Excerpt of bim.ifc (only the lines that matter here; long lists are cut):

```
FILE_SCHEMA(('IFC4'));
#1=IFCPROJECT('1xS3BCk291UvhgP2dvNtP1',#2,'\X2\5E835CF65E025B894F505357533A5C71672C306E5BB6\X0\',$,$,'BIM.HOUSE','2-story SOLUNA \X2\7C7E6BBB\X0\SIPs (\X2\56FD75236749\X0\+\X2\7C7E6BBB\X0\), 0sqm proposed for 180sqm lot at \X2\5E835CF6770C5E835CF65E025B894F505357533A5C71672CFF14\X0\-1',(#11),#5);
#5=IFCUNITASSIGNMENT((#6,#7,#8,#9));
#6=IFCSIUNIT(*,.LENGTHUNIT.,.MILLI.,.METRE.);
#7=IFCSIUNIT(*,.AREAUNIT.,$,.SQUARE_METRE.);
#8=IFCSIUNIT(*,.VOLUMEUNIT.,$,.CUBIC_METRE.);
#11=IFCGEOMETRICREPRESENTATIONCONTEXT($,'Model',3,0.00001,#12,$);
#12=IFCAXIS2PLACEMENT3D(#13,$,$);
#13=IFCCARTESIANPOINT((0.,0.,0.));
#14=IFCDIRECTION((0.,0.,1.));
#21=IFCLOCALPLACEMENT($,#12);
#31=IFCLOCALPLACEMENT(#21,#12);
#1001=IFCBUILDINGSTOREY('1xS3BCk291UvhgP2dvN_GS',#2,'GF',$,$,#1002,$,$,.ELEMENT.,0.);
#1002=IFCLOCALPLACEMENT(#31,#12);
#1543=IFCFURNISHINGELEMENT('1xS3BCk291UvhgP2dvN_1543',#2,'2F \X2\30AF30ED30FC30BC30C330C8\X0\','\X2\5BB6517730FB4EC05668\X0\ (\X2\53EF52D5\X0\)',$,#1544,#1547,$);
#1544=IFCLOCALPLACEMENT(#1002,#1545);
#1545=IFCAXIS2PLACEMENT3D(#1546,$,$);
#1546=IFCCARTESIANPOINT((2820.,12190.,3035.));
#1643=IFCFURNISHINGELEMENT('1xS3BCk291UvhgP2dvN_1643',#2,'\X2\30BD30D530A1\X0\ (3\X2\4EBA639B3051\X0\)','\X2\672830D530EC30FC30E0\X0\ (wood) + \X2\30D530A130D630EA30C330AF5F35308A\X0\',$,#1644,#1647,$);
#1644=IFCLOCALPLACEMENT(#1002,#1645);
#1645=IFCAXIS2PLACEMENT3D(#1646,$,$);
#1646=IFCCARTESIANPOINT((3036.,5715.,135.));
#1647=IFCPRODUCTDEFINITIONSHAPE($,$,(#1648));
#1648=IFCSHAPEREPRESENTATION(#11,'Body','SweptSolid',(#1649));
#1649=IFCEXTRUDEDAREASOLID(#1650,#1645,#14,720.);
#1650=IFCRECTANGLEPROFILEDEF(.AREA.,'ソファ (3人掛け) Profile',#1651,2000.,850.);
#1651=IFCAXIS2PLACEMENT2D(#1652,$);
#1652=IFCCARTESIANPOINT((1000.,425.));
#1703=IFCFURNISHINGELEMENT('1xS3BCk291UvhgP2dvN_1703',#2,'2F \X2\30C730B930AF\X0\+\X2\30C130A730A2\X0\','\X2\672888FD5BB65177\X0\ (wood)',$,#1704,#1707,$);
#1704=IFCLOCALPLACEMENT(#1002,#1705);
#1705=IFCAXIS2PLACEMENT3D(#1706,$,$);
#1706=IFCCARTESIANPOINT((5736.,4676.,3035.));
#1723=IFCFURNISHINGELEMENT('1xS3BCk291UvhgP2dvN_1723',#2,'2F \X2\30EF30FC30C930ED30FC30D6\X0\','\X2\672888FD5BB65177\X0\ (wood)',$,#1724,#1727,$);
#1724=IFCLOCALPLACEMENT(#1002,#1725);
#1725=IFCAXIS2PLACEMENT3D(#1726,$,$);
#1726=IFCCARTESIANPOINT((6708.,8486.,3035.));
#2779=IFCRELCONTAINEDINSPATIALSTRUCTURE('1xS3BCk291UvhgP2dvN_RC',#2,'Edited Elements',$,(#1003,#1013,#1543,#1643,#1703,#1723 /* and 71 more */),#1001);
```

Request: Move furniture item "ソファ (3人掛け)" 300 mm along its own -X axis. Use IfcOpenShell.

```python
import ifcopenshell
import ifcopenshell.api.geometry
import ifcopenshell.util.placement
import ifcopenshell.util.unit

model = ifcopenshell.open("bim.ifc")
unit_scale = ifcopenshell.util.unit.calculate_unit_scale(model)

item = model.by_id(1643)
matrix = ifcopenshell.util.placement.get_local_placement(item.ObjectPlacement)
matrix[:3, 3] -= matrix[:3, 0] * 0.3 / unit_scale
ifcopenshell.api.geometry.edit_object_placement(model, product=item, matrix=matrix, is_si=False)

print(ifcopenshell.util.placement.get_local_placement(item.ObjectPlacement).round(3) + 0.0)

model.write("bim_rev.ifc")
```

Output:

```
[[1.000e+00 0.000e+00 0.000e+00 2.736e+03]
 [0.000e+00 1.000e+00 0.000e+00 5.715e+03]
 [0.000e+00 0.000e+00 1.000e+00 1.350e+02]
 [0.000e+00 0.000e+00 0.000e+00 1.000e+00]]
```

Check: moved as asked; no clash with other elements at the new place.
